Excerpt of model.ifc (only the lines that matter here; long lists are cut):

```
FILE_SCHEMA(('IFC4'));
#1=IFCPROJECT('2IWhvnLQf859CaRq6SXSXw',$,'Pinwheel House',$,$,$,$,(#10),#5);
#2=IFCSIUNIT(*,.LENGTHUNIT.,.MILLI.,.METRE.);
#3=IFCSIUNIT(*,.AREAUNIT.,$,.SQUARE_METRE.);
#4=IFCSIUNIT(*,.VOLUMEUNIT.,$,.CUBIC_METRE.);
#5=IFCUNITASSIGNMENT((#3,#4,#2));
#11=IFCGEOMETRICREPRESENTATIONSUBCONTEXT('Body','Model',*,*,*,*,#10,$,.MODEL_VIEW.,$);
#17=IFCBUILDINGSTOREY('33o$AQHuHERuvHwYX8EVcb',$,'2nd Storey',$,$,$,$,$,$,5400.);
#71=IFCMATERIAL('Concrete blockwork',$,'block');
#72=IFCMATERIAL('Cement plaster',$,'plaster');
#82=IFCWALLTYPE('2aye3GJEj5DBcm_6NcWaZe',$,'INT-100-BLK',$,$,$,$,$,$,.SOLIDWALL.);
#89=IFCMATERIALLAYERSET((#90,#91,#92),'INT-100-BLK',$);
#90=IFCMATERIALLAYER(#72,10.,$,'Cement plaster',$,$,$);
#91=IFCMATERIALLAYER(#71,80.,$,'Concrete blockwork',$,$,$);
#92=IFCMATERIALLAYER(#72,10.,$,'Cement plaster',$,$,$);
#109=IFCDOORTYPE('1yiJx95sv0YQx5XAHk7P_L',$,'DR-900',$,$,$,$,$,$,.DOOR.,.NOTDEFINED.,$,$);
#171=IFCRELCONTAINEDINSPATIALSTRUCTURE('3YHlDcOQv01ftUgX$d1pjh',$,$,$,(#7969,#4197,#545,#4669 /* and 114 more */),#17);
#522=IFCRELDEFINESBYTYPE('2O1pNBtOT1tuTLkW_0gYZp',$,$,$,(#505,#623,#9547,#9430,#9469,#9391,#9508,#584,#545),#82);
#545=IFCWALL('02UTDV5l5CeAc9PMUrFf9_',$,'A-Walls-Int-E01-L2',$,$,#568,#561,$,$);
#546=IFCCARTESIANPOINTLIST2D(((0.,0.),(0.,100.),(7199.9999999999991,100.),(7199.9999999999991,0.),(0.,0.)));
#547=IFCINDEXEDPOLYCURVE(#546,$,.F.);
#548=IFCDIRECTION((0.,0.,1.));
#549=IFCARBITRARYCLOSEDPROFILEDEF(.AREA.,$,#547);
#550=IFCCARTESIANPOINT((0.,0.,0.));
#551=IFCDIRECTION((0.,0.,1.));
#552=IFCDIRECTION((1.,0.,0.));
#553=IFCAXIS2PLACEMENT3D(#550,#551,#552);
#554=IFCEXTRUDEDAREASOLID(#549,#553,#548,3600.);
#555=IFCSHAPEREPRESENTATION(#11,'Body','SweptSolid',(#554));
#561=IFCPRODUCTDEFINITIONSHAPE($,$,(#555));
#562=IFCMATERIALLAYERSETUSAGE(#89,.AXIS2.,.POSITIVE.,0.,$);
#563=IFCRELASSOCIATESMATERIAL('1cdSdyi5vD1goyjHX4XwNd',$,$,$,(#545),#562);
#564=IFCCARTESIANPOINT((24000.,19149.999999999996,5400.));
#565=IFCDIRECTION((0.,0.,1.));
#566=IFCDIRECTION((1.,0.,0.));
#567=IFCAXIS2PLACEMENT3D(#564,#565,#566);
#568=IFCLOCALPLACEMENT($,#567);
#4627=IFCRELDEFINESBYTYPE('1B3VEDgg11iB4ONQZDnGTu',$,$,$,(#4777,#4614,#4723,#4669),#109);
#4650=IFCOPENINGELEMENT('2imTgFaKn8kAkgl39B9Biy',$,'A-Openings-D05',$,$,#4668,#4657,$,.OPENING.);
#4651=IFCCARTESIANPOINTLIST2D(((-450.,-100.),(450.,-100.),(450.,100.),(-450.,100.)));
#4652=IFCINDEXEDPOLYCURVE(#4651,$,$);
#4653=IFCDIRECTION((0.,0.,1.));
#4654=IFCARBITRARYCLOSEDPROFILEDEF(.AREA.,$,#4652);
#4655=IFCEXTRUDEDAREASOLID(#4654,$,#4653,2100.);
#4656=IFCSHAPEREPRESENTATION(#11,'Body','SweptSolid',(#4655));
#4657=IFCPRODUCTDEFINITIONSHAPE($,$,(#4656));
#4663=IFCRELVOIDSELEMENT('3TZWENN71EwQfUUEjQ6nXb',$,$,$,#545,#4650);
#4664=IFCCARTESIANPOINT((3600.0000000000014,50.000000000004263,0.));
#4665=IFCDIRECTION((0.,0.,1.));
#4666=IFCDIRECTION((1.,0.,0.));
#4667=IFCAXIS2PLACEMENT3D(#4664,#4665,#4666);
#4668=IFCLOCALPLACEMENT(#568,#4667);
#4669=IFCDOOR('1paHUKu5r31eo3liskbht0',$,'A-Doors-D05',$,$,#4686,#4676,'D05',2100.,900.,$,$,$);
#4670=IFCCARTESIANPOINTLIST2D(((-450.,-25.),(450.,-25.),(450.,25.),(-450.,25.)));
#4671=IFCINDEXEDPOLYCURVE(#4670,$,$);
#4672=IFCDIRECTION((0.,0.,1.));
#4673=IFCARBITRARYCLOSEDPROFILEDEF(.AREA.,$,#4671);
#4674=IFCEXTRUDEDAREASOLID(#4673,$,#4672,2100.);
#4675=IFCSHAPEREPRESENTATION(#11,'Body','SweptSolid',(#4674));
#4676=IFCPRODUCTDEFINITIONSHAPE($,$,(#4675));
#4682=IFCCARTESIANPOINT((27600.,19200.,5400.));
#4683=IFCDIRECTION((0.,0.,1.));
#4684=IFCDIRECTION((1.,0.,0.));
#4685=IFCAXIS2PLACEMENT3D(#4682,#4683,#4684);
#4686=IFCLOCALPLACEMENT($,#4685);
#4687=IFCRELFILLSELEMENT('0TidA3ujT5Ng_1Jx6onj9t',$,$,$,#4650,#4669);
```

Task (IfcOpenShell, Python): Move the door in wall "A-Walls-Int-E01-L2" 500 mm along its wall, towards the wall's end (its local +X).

```python
import ifcopenshell
import ifcopenshell.api.geometry
import ifcopenshell.util.placement
import ifcopenshell.util.unit

model = ifcopenshell.open("model.ifc")
unit_scale = ifcopenshell.util.unit.calculate_unit_scale(model)

door = model.by_id(4669)
opening = door.FillsVoids[0].RelatingOpeningElement
wall = opening.VoidsElements[0].RelatingBuildingElement

wall_matrix = ifcopenshell.util.placement.get_local_placement(wall.ObjectPlacement)
shift = wall_matrix[:3, 0] * 0.5 / unit_scale
before = ifcopenshell.util.placement.get_local_placement(door.ObjectPlacement)[:3, 3].copy()

# The door is not placed relative to its opening, so move both.
for product in (opening, door):
    matrix = ifcopenshell.util.placement.get_local_placement(product.ObjectPlacement)
    matrix[:3, 3] += shift
    ifcopenshell.api.geometry.edit_object_placement(model, product=product, matrix=matrix, is_si=False)

after = ifcopenshell.util.placement.get_local_placement(door.ObjectPlacement)[:3, 3]
print("door moved by", (after - before).round(3) + 0.0)

model.write("model_v2.ifc")
```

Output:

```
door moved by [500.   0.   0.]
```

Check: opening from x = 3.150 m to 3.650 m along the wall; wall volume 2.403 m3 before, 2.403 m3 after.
